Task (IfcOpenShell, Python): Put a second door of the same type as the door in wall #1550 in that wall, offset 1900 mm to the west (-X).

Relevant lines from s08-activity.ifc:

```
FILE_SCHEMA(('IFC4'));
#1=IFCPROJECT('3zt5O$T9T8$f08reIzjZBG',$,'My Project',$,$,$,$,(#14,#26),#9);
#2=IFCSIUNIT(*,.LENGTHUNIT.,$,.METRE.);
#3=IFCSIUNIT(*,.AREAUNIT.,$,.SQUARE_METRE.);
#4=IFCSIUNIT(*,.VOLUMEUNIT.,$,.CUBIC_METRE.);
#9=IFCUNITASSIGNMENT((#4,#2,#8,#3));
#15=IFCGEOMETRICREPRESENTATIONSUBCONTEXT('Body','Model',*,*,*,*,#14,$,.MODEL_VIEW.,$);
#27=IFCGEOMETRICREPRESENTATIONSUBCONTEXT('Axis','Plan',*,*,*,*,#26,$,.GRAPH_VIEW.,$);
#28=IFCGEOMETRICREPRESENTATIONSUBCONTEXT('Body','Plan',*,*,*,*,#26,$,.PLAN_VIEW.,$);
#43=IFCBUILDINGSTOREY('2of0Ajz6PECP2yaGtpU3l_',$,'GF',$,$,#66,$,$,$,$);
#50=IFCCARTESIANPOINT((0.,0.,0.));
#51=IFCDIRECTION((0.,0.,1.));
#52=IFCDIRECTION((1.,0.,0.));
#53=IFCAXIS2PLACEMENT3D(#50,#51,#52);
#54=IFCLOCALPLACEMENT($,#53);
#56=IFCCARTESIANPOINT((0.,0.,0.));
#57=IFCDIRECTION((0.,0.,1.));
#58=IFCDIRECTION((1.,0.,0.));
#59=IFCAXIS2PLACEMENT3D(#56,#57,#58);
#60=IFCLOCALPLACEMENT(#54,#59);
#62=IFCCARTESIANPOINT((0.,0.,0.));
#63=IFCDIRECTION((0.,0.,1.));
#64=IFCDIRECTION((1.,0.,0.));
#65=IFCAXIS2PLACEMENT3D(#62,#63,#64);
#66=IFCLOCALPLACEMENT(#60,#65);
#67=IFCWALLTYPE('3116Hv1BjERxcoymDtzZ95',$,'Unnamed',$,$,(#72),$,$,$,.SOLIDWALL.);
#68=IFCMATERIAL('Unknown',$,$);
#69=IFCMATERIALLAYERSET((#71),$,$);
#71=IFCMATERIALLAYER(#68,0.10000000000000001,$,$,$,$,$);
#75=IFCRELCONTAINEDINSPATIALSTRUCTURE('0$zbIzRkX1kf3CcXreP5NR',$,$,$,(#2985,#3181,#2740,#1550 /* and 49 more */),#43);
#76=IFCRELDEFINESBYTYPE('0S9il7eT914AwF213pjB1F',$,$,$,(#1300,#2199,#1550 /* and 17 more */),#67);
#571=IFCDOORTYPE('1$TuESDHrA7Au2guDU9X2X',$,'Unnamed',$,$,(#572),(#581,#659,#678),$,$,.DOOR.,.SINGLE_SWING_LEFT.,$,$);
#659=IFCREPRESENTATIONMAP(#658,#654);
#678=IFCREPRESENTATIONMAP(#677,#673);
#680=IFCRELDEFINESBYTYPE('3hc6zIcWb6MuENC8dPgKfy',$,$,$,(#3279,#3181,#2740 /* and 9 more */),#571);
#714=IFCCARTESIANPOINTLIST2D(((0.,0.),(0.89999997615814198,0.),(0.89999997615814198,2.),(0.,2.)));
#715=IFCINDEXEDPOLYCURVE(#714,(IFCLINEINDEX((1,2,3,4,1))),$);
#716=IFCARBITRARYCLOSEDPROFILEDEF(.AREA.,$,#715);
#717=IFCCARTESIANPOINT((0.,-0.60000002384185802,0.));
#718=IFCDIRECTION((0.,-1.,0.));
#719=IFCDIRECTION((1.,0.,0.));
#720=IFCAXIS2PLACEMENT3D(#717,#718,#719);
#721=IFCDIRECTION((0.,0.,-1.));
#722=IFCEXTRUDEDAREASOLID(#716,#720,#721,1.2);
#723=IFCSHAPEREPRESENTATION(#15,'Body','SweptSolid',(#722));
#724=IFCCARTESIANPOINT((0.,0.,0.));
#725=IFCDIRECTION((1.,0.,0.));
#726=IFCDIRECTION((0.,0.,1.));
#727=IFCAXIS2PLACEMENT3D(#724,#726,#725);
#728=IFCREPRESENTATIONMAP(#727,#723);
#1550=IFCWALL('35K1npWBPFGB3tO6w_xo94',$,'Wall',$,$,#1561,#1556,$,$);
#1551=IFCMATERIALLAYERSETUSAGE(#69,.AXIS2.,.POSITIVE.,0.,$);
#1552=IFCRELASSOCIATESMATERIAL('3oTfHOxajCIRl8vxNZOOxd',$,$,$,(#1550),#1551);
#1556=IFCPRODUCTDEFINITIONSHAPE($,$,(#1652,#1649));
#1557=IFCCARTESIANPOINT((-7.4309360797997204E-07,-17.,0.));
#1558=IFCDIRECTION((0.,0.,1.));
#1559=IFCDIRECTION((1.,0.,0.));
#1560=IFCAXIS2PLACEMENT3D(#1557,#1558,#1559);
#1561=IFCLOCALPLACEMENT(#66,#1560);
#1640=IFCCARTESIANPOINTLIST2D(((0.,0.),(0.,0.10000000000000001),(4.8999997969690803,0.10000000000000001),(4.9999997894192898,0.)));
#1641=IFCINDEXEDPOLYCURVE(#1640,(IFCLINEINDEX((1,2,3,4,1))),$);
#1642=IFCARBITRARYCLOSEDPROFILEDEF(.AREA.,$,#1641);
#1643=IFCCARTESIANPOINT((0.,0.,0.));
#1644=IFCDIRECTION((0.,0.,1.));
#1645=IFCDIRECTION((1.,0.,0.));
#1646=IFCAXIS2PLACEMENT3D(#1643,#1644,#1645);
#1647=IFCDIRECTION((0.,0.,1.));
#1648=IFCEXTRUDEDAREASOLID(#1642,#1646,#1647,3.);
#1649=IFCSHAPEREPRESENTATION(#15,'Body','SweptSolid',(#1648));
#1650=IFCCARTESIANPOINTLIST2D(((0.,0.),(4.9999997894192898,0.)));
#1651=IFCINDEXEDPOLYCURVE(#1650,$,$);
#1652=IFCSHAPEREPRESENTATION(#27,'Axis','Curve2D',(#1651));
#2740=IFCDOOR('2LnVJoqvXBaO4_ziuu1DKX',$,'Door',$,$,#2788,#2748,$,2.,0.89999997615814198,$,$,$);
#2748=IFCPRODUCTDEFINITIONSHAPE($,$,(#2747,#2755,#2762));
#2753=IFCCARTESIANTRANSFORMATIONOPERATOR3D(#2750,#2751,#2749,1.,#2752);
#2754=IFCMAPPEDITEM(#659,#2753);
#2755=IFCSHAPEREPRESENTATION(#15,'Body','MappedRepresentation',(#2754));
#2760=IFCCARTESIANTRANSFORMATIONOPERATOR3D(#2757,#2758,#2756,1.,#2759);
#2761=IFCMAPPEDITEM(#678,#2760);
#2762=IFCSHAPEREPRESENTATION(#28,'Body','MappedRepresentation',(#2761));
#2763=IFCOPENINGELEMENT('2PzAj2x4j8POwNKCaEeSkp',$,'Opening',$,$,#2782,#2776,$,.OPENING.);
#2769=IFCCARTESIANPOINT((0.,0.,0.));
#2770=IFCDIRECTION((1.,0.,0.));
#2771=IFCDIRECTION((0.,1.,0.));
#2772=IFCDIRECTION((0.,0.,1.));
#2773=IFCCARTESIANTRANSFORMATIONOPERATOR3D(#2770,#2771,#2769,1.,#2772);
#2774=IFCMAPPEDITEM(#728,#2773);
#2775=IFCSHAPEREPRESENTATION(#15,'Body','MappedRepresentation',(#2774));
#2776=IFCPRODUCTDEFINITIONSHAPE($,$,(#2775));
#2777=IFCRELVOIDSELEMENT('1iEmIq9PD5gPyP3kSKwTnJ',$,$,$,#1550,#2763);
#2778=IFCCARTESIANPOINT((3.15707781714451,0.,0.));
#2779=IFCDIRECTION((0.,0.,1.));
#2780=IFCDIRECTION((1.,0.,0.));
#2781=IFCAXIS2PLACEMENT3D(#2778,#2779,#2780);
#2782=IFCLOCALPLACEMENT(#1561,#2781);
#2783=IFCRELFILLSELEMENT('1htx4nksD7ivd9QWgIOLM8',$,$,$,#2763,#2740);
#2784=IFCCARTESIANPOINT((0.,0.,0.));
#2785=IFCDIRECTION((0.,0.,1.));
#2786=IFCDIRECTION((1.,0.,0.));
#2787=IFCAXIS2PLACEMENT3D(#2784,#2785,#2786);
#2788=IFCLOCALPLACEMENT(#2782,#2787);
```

```python
import ifcopenshell
import ifcopenshell.api.feature
import ifcopenshell.api.geometry
import ifcopenshell.api.root
import ifcopenshell.geom
import ifcopenshell.util.element
import ifcopenshell.util.placement
import ifcopenshell.util.shape
import ifcopenshell.util.unit

model = ifcopenshell.open("s08-activity.ifc")
unit_scale = ifcopenshell.util.unit.calculate_unit_scale(model)
settings = ifcopenshell.geom.settings()


def volume(element):
    """Net volume in cubic metres, openings subtracted."""
    shape = ifcopenshell.geom.create_shape(settings, element)
    return ifcopenshell.util.shape.get_volume(shape.geometry)


door = model.by_guid("2LnVJoqvXBaO4_ziuu1DKX")
opening = door.FillsVoids[0].RelatingOpeningElement
wall = opening.VoidsElements[0].RelatingBuildingElement
before = volume(wall)
shift = ifcopenshell.util.placement.get_local_placement(wall.ObjectPlacement)[:3, 0] * -1.9 / unit_scale

# copy_class copies the void relationship, type, container and properties, but no geometry.
new_opening = ifcopenshell.api.root.copy_class(model, product=opening)
new_opening.Representation = ifcopenshell.util.element.copy_deep(
    model, opening.Representation, exclude=["IfcGeometricRepresentationContext", "IfcRepresentationMap"]
)
new_door = ifcopenshell.api.root.copy_class(model, product=door)
new_door.Representation = ifcopenshell.util.element.copy_deep(
    model, door.Representation, exclude=["IfcGeometricRepresentationContext", "IfcRepresentationMap"]
)
ifcopenshell.api.feature.add_filling(model, opening=new_opening, element=new_door)

for old, new in ((opening, new_opening), (door, new_door)):
    matrix = ifcopenshell.util.placement.get_local_placement(old.ObjectPlacement)
    matrix[:3, 3] += shift
    ifcopenshell.api.geometry.edit_object_placement(model, product=new, matrix=matrix, is_si=False)

after = volume(wall)

print(f"wall volume {before:.3f} -> {after:.3f} m3")

model.write("s08-activity_v2.ifc")
```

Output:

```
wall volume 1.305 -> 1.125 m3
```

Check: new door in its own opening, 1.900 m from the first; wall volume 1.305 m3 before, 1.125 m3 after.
